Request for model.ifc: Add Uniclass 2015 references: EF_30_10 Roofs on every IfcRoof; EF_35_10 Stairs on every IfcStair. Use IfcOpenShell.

First a look at what the model holds.

```python
import ifcopenshell

model = ifcopenshell.open("model.ifc")
print(model.schema)
print("classifications:", [c.Name for c in model.by_type("IfcClassification")])
for ifc_class in ("IfcDoor", "IfcRoof", "IfcStair", "IfcWall", "IfcWindow"):
    print(ifc_class, len(model.by_type(ifc_class)))
```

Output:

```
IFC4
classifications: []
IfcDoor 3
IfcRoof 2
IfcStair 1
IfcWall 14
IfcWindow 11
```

```python
import ifcopenshell
import ifcopenshell.api.classification

model = ifcopenshell.open("model.ifc")

system = ifcopenshell.api.classification.add_classification(model, classification="Uniclass 2015")

codes = {
    "IfcRoof": ("EF_30_10", "Roofs"),
    "IfcStair": ("EF_35_10", "Stairs"),
}
for ifc_class, (code, name) in codes.items():
    products = model.by_type(ifc_class)
    ifcopenshell.api.classification.add_reference(
        model, products=products, classification=system, identification=code, name=name
    )
    print(code, len(products))

model.write("model_updated.ifc")
```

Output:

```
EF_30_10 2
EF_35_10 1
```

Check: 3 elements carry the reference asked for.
